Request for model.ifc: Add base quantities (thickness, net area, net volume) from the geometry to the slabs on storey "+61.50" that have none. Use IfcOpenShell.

First a look at what the model holds.

```python
import ifcopenshell
import ifcopenshell.util.element
import ifcopenshell.util.unit

model = ifcopenshell.open("model.ifc")
print(model.schema)
for unit_type in ("LENGTHUNIT", "AREAUNIT", "VOLUMEUNIT"):
    print(unit_type, ifcopenshell.util.unit.calculate_unit_scale(model, unit_type))
storey = next(s for s in model.by_type("IfcBuildingStorey") if s.Name == "+61.50")
slabs = [e for e in ifcopenshell.util.element.get_decomposition(storey) if e.is_a("IfcSlab")]
for e in sorted(slabs, key=lambda e: e.id()):
    print(e.id(), e.is_a(), e.Name, list(ifcopenshell.util.element.get_psets(e, qtos_only=True)), sep=" | ")
```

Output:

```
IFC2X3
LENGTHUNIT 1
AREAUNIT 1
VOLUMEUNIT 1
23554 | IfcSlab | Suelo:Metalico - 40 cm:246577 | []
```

```python
import ifcopenshell
import ifcopenshell.api.pset
import ifcopenshell.geom
import ifcopenshell.util.element
import ifcopenshell.util.shape
import ifcopenshell.util.unit

model = ifcopenshell.open("model.ifc")
unit_scale = ifcopenshell.util.unit.calculate_unit_scale(model)
area_scale = ifcopenshell.util.unit.calculate_unit_scale(model, "AREAUNIT")
volume_scale = ifcopenshell.util.unit.calculate_unit_scale(model, "VOLUMEUNIT")
settings = ifcopenshell.geom.settings()

storey = next(s for s in model.by_type("IfcBuildingStorey") if s.Name == "+61.50")
slabs = [e for e in ifcopenshell.util.element.get_decomposition(storey) if e.is_a("IfcSlab")]

for e in sorted(slabs, key=lambda e: e.id()):
    if ifcopenshell.util.element.get_psets(e, qtos_only=True, should_inherit=False):
        continue
    # Geometry comes back in metres, in the element's own axes.
    shape = ifcopenshell.geom.create_shape(settings, e)
    values = {
        "Width": ifcopenshell.util.shape.get_z(shape.geometry) / unit_scale,
        "NetArea": ifcopenshell.util.shape.get_footprint_area(shape.geometry) / area_scale,
        "NetVolume": ifcopenshell.util.shape.get_volume(shape.geometry) / volume_scale,
    }
    qto = ifcopenshell.api.pset.add_qto(model, product=e, name="BaseQuantities")
    ifcopenshell.api.pset.edit_qto(model, qto=qto, properties=values)
    print(e.id(), {k: round(v, 3) for k, v in values.items()})

model.write("model_rev.ifc")
```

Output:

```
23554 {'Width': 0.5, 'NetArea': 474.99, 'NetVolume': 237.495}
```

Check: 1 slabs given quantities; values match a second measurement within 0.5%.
